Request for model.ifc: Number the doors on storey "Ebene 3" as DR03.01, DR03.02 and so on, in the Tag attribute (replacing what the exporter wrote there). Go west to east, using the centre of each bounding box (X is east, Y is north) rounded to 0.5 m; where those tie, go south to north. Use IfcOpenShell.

First a look at what the model holds.

```python
import ifcopenshell
import ifcopenshell.util.element
import ifcopenshell.util.placement

model = ifcopenshell.open("model.ifc")
print(model.schema)
storey = next(s for s in model.by_type("IfcBuildingStorey") if s.Name == "Ebene 3")
doors = [e for e in ifcopenshell.util.element.get_decomposition(storey) if e.is_a("IfcDoor")]
for e in sorted(doors, key=lambda e: e.id()):
    origin = ifcopenshell.util.placement.get_local_placement(e.ObjectPlacement)[:3, 3]
    print(e.id(), e.Tag, e.Name, origin.round(2) + 0.0, sep=" | ")
```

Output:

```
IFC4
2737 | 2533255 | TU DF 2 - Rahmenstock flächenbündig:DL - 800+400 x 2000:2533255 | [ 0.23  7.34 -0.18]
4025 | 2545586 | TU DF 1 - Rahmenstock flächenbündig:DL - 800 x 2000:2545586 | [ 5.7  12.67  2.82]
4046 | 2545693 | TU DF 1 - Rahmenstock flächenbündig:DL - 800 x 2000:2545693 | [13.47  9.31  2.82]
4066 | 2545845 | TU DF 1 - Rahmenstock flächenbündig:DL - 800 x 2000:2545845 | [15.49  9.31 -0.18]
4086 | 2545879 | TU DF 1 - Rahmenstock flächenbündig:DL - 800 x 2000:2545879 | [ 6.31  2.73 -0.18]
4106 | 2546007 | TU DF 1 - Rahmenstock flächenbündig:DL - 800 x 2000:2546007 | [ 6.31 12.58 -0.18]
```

```python
import ifcopenshell
import ifcopenshell.geom
import ifcopenshell.util.element
import ifcopenshell.util.shape

model = ifcopenshell.open("model.ifc")
settings = ifcopenshell.geom.settings()
settings.set("use-world-coords", True)


def centre(element):
    shape = ifcopenshell.geom.create_shape(settings, element)
    return ifcopenshell.util.shape.get_bbox_centroid(shape.geometry)


storey = next(s for s in model.by_type("IfcBuildingStorey") if s.Name == "Ebene 3")
doors = [e for e in ifcopenshell.util.element.get_decomposition(storey) if e.is_a("IfcDoor")]

# Insertion points can sit at a corner or the storey origin, so sort by the geometry (in metres).
centres = {e: centre(e) for e in doors}
doors.sort(key=lambda e: (round(centres[e][0] / 0.5), centres[e][1]))

for i, e in enumerate(doors, start=1):
    number = f"DR03.{i:02d}"
    e.Tag = number
    print(e.id(), number)

model.write("model_rev.ifc")
```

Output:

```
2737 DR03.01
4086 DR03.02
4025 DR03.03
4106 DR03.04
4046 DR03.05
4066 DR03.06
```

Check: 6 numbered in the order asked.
